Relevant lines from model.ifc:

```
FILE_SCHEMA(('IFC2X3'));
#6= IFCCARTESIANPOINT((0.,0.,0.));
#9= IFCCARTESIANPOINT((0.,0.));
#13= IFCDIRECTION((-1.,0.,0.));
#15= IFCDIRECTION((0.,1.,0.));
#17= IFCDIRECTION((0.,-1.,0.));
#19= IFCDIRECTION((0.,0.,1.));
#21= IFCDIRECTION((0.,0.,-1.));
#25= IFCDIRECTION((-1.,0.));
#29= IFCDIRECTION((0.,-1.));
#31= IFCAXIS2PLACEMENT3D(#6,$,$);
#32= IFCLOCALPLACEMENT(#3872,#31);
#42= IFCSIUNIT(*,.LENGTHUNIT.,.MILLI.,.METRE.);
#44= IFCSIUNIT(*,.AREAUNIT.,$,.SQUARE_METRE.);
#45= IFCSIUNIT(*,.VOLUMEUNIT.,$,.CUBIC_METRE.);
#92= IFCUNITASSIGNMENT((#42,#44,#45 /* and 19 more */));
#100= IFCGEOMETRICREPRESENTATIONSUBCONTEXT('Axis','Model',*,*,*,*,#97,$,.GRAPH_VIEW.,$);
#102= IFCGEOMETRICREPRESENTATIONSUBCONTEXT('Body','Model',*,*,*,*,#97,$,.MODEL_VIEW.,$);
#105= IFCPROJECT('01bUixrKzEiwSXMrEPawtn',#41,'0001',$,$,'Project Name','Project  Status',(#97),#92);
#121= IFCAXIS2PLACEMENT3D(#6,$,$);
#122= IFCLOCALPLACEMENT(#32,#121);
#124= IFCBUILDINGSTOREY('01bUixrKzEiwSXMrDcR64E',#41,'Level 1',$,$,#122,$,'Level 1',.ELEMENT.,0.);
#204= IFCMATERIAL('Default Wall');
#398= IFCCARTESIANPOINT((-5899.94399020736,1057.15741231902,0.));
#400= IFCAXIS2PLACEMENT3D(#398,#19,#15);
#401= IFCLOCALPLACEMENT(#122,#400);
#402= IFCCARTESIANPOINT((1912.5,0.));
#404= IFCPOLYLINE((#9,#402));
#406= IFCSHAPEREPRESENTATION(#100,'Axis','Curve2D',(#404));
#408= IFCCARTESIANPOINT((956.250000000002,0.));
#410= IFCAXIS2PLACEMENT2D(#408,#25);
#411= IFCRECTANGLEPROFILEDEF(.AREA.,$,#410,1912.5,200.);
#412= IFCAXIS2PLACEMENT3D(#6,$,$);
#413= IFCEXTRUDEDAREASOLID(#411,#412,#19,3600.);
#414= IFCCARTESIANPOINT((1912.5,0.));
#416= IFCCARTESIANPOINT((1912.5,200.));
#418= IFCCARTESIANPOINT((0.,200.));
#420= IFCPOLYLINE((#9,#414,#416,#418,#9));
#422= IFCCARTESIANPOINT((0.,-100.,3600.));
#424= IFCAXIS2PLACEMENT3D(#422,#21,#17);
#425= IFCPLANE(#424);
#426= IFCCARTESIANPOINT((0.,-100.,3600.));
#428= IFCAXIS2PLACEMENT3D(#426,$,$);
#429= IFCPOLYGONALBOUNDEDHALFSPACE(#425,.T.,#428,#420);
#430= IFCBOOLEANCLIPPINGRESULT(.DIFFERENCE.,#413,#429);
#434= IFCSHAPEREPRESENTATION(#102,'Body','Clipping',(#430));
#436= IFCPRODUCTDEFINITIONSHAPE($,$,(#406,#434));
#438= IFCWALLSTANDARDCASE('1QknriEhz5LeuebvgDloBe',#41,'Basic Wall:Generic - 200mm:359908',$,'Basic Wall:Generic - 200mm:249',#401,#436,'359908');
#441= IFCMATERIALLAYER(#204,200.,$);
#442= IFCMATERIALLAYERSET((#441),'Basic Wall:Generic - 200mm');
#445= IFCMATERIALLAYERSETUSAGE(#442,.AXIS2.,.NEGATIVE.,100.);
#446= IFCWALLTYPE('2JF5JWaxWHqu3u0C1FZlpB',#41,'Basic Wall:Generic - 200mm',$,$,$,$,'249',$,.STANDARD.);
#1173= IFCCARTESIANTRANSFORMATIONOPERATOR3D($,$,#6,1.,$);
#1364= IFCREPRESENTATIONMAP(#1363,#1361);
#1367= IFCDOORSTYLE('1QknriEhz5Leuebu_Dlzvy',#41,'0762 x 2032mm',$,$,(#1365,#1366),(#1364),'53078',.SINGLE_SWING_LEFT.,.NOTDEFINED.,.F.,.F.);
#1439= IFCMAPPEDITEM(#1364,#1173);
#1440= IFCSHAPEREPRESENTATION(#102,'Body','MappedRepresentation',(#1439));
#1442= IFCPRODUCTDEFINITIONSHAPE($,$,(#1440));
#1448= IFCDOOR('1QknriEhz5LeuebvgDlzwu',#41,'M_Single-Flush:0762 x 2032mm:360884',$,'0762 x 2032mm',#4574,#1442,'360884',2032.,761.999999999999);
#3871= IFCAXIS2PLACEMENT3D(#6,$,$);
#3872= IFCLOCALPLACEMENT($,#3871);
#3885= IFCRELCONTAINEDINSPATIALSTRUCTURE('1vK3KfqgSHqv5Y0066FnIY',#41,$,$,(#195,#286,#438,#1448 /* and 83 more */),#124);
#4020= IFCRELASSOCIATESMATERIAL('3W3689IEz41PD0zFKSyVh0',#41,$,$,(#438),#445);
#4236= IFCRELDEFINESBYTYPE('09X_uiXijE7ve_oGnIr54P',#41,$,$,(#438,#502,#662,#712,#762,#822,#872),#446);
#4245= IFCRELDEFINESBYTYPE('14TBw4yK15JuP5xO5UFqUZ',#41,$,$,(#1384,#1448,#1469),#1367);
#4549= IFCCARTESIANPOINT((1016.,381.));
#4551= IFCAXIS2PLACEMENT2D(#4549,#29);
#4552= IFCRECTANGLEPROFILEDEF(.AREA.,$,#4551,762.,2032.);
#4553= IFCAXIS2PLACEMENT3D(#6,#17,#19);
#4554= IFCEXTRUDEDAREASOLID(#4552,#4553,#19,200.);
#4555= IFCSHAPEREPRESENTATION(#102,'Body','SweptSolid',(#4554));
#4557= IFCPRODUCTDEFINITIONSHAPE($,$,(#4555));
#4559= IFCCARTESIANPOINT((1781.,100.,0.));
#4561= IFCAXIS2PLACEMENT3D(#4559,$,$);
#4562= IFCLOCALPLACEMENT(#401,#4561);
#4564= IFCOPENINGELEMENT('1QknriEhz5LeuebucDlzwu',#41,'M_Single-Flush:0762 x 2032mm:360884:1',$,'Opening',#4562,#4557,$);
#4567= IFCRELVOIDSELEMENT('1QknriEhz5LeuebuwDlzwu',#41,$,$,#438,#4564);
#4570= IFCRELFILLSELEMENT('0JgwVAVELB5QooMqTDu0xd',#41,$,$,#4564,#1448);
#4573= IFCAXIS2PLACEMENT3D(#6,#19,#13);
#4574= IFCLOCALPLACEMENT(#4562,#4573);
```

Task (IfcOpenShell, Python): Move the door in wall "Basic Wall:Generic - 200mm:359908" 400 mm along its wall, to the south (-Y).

```python
import ifcopenshell
import ifcopenshell.api.geometry
import ifcopenshell.util.placement

model = ifcopenshell.open("model.ifc")

door = model.by_guid("1QknriEhz5LeuebvgDlzwu")
opening = door.FillsVoids[0].RelatingOpeningElement
wall = opening.VoidsElements[0].RelatingBuildingElement

wall_matrix = ifcopenshell.util.placement.get_local_placement(wall.ObjectPlacement)
shift = wall_matrix[:3, 0] * -400.0
before = ifcopenshell.util.placement.get_local_placement(door.ObjectPlacement)[:3, 3].copy()

# The door is placed relative to its opening, so it follows when the opening moves.
matrix = ifcopenshell.util.placement.get_local_placement(opening.ObjectPlacement)
matrix[:3, 3] += shift
ifcopenshell.api.geometry.edit_object_placement(
    model, product=opening, matrix=matrix, is_si=False, should_transform_children=True
)

after = ifcopenshell.util.placement.get_local_placement(door.ObjectPlacement)[:3, 3]
print("door moved by", (after - before).round(3) + 0.0)

model.write("model_updated.ifc")
```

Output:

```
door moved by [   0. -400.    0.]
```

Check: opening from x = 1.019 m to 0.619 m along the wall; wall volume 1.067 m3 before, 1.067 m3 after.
